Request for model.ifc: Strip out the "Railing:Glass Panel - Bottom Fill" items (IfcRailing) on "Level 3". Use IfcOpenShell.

First a look at what the model holds.

```python
import ifcopenshell
import ifcopenshell.util.element

model = ifcopenshell.open("model.ifc")
print(model.schema)
storey = next(s for s in model.by_type("IfcBuildingStorey") if s.Name == "Level 3")
railings = [e for e in ifcopenshell.util.element.get_decomposition(storey) if e.is_a("IfcRailing")]
seen = {}
for e in railings:
    element_type = ifcopenshell.util.element.get_type(e)
    name = element_type.Name if element_type not in (None, e) else None
    seen[name] = seen.get(name, 0) + 1
for name, count in sorted(seen.items(), key=str):
    print(count, "x", name)
```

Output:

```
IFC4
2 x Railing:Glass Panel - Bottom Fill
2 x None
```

```python
import ifcopenshell
import ifcopenshell.api.root
import ifcopenshell.util.element

model = ifcopenshell.open("model.ifc")

storey = next(s for s in model.by_type("IfcBuildingStorey") if s.Name == "Level 3")
railings = [e for e in ifcopenshell.util.element.get_decomposition(storey) if e.is_a("IfcRailing")]
targets = [e for e in railings if (t := ifcopenshell.util.element.get_type(e)) not in (None, e) and t.Name == "Railing:Glass Panel - Bottom Fill"]

for e in targets:
    ifcopenshell.api.root.remove_product(model, product=e)
print(len(targets), "removed")

model.write("model_rev.ifc")
```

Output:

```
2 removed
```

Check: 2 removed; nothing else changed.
